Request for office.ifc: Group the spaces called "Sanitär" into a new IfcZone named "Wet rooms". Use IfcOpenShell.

First a look at what the model holds.

```python
import ifcopenshell

model = ifcopenshell.open("office.ifc")
print(model.schema)
seen = {}
for space in model.by_type("IfcSpace"):
    seen[space.LongName] = seen.get(space.LongName, 0) + 1
for name, count in sorted(seen.items(), key=str):
    print(count, "x", name)
print("zones:", [z.Name for z in model.by_type("IfcZone")][:20])
```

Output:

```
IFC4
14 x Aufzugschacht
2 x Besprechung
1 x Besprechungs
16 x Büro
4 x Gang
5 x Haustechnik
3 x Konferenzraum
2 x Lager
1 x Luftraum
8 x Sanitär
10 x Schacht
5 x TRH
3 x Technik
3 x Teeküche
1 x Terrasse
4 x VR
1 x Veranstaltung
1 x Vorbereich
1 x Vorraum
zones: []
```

```python
import ifcopenshell
import ifcopenshell.api.group
import ifcopenshell.api.root

model = ifcopenshell.open("office.ifc")

names = {"Sanitär"}
spaces = [s for s in model.by_type("IfcSpace") if s.LongName in names]

zone = ifcopenshell.api.root.create_entity(model, ifc_class="IfcZone", name="Wet rooms")
ifcopenshell.api.group.assign_group(model, products=spaces, group=zone)
print(len(spaces), "spaces in", zone.Name)

model.write("office_updated.ifc")
```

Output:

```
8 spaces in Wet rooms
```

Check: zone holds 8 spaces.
